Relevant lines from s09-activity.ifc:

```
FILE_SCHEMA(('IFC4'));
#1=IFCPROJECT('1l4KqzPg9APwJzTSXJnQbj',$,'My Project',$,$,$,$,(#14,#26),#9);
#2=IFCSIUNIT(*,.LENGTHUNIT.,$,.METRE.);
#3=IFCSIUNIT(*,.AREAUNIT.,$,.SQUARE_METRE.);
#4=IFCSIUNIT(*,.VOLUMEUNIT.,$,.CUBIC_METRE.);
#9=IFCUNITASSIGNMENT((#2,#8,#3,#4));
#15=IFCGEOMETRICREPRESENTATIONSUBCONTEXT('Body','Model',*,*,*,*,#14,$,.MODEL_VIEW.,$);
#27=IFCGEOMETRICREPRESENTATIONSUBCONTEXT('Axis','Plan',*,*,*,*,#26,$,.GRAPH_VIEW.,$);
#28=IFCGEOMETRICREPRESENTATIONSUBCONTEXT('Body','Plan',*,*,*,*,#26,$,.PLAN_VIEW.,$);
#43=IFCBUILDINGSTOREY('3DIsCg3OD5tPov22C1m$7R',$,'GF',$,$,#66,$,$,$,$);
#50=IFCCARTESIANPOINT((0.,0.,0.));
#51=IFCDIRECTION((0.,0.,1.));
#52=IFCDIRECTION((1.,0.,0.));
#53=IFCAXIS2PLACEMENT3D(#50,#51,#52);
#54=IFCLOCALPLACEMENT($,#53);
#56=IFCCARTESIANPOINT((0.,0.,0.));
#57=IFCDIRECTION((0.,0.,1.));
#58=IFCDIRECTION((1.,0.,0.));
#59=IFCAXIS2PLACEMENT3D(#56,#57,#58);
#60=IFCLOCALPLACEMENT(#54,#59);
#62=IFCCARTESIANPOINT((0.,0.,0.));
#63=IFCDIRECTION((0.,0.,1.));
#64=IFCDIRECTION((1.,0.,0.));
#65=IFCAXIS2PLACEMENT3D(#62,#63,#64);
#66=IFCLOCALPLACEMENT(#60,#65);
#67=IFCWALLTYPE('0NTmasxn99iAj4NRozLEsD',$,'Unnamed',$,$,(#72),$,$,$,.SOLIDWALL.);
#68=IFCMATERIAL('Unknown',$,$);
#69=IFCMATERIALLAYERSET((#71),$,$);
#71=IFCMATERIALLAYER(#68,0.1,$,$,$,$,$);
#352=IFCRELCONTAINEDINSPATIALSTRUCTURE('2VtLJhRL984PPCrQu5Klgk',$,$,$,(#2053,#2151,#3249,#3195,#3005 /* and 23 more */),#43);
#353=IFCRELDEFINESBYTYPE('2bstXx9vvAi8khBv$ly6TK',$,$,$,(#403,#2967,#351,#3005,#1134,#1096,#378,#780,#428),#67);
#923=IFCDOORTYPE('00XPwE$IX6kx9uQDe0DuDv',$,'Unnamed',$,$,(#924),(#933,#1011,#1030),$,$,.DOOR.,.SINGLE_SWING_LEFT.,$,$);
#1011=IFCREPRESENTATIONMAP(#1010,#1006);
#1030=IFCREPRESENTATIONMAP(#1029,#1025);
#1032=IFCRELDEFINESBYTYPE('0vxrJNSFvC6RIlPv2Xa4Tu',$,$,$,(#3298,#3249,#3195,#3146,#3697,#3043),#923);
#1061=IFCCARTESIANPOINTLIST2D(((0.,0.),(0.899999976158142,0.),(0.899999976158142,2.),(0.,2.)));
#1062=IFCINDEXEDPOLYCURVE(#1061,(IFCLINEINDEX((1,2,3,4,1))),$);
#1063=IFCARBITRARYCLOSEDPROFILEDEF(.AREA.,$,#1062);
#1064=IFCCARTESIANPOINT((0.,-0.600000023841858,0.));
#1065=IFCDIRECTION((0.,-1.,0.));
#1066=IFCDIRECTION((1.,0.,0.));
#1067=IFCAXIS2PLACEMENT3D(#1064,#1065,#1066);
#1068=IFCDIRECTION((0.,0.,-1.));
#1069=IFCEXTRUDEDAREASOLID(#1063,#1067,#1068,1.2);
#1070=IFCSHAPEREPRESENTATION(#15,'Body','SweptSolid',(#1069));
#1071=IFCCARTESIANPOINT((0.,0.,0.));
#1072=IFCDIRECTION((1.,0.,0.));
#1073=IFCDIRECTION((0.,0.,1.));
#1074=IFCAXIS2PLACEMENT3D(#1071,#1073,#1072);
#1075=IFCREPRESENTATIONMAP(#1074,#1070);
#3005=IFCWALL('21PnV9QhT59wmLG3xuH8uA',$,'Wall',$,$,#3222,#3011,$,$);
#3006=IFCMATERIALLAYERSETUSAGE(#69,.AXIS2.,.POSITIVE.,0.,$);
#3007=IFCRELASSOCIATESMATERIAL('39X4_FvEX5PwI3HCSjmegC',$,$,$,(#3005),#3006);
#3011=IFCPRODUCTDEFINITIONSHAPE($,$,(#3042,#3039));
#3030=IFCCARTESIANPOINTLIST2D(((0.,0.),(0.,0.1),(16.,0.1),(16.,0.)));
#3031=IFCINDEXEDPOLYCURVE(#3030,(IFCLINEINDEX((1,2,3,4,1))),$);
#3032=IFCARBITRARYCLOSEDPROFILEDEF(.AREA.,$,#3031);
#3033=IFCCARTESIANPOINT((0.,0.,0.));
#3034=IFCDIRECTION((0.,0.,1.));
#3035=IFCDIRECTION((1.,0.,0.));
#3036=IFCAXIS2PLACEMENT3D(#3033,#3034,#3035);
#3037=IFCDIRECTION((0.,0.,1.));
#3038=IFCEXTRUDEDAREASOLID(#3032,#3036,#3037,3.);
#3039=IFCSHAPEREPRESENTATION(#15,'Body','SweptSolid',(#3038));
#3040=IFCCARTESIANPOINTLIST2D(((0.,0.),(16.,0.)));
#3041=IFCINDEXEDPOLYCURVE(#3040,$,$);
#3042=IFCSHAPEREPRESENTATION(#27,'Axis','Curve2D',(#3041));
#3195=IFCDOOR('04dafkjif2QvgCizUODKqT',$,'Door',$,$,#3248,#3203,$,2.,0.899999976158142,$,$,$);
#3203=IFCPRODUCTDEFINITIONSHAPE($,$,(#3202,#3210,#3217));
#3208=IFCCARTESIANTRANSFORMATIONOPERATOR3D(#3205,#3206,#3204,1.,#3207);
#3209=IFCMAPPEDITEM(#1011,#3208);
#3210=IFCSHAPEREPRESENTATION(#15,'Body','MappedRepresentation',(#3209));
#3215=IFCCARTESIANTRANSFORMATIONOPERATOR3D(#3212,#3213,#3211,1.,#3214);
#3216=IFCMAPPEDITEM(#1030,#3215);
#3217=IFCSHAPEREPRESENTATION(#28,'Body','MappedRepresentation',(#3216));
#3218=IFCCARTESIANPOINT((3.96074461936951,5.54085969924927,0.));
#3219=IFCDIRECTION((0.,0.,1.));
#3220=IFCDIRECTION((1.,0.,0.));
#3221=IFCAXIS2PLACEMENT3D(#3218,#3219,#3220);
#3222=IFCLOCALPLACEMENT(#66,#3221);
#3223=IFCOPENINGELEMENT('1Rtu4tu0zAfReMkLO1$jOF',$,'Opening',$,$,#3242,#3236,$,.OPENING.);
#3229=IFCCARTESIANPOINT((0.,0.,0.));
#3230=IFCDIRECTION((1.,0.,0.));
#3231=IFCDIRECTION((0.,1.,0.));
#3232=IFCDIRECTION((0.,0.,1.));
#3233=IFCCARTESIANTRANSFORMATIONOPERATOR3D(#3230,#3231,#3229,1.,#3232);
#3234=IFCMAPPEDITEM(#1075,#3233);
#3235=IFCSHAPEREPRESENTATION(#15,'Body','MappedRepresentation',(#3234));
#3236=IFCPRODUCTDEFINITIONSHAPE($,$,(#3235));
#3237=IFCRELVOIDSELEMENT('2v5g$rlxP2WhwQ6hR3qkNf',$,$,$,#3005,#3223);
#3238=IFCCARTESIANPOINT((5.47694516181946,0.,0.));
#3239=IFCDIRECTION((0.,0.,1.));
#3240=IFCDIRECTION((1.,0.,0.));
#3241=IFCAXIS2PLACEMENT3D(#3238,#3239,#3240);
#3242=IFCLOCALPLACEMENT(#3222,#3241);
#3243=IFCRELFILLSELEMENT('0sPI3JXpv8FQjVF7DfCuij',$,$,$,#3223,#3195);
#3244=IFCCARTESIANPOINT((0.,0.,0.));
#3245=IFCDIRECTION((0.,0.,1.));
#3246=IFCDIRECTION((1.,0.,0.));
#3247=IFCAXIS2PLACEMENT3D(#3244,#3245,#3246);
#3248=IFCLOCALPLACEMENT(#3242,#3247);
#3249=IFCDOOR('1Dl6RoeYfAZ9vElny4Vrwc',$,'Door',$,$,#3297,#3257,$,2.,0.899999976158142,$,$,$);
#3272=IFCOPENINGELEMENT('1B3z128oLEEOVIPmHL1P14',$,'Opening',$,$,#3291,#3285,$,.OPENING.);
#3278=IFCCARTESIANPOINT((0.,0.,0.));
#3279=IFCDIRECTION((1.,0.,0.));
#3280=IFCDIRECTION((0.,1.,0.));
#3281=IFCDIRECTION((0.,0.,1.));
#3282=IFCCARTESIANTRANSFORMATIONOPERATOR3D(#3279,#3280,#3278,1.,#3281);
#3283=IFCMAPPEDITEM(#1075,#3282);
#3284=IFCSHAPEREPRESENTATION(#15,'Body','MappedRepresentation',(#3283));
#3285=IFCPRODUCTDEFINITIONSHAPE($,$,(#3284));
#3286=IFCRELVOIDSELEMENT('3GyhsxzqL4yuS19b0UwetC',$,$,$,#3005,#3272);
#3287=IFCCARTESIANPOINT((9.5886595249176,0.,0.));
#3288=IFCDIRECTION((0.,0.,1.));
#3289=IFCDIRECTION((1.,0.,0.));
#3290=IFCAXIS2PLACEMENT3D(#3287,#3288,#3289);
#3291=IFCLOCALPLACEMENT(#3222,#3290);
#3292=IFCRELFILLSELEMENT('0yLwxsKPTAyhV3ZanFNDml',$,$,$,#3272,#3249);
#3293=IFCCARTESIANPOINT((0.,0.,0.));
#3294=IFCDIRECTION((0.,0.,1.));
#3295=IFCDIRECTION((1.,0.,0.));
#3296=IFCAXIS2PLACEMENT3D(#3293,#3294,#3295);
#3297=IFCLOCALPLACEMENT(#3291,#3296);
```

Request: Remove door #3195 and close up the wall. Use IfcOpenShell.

```python
import ifcopenshell
import ifcopenshell.api.feature
import ifcopenshell.api.root
import ifcopenshell.geom
import ifcopenshell.util.shape

model = ifcopenshell.open("s09-activity.ifc")
settings = ifcopenshell.geom.settings()


def volume(element):
    """Net volume in cubic metres, openings subtracted."""
    shape = ifcopenshell.geom.create_shape(settings, element)
    return ifcopenshell.util.shape.get_volume(shape.geometry)


door = model.by_guid("04dafkjif2QvgCizUODKqT")
opening = door.FillsVoids[0].RelatingOpeningElement
wall = opening.VoidsElements[0].RelatingBuildingElement
before = volume(wall)

ifcopenshell.api.root.remove_product(model, product=door)
ifcopenshell.api.feature.remove_feature(model, feature=opening)

after = volume(wall)

print(f"wall volume {before:.3f} -> {after:.3f} m3")

model.write("s09-activity_rev.ifc")
```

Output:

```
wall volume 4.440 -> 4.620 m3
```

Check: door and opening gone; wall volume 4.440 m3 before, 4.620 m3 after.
